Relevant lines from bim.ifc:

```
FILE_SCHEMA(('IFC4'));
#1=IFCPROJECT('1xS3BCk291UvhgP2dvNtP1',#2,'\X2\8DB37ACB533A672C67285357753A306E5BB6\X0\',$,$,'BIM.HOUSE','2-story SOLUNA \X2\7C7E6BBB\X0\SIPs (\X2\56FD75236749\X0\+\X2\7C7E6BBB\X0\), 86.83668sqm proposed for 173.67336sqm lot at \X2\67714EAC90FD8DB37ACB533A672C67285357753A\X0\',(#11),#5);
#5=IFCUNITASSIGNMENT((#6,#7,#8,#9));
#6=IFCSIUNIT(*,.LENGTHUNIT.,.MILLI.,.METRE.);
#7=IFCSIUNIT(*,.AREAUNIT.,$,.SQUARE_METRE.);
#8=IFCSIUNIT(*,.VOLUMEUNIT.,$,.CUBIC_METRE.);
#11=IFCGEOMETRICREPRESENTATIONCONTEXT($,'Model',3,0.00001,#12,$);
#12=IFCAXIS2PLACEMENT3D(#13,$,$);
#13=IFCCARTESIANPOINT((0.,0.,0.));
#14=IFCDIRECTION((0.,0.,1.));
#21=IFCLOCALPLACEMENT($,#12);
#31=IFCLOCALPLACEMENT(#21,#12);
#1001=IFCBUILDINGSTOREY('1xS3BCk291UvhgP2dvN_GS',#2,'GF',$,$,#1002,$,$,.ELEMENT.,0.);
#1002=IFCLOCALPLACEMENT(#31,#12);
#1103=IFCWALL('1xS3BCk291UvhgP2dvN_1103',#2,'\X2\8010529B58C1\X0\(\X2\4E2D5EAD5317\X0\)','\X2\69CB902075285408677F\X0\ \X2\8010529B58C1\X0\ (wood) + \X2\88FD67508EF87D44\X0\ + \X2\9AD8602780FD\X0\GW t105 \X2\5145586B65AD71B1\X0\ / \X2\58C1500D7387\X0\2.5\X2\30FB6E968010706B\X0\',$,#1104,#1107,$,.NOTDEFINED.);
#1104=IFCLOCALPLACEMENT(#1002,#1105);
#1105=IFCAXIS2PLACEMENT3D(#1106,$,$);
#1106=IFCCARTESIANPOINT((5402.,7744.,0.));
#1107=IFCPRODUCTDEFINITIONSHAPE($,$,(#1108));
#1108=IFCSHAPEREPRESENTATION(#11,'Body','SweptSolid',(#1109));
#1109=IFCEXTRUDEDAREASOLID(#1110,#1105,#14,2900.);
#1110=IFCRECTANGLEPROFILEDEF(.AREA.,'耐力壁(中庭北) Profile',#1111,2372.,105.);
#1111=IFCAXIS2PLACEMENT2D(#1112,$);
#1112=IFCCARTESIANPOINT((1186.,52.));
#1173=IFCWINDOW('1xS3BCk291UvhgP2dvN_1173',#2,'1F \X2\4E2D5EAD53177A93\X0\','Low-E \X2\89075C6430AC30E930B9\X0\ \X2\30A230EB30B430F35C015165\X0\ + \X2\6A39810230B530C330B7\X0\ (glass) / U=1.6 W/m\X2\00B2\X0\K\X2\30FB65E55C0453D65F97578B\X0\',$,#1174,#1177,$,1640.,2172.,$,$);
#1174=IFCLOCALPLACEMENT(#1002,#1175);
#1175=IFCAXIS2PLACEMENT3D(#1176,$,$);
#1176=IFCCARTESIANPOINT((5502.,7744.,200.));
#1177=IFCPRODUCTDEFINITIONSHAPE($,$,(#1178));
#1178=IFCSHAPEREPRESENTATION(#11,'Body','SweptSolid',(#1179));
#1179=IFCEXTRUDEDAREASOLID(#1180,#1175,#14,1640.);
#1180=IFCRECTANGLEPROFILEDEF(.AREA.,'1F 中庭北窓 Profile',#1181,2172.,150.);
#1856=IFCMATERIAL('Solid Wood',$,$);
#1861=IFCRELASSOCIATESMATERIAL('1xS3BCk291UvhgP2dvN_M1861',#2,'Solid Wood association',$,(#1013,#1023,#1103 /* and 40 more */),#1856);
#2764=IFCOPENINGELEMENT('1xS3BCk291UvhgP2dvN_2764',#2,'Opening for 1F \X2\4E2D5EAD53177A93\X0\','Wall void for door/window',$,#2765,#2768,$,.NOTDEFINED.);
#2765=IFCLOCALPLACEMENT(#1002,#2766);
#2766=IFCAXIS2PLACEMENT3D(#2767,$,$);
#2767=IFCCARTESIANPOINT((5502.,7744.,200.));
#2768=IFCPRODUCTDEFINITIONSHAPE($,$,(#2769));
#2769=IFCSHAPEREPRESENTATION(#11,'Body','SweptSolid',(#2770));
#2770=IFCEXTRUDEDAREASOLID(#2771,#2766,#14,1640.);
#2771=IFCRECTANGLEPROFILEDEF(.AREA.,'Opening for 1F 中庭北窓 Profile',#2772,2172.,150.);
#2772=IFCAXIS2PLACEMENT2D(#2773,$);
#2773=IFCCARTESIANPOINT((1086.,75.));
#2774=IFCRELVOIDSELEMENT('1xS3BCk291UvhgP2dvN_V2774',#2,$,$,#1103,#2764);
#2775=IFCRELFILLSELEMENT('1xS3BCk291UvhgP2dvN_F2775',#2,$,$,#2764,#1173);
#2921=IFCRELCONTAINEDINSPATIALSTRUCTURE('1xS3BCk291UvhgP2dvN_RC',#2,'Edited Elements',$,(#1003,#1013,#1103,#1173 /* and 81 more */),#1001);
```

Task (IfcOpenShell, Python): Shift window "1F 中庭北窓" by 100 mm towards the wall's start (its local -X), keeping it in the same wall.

```python
import ifcopenshell
import ifcopenshell.api.geometry
import ifcopenshell.util.placement

model = ifcopenshell.open("bim.ifc")

window = model.by_guid("1xS3BCk291UvhgP2dvN_1173")
opening = window.FillsVoids[0].RelatingOpeningElement
wall = opening.VoidsElements[0].RelatingBuildingElement

wall_matrix = ifcopenshell.util.placement.get_local_placement(wall.ObjectPlacement)
shift = wall_matrix[:3, 0] * -100.0
before = ifcopenshell.util.placement.get_local_placement(window.ObjectPlacement)[:3, 3].copy()

# The window is not placed relative to its opening, so move both.
for product in (opening, window):
    matrix = ifcopenshell.util.placement.get_local_placement(product.ObjectPlacement)
    matrix[:3, 3] += shift
    ifcopenshell.api.geometry.edit_object_placement(model, product=product, matrix=matrix, is_si=False)

after = ifcopenshell.util.placement.get_local_placement(window.ObjectPlacement)[:3, 3]
print("window moved by", (after - before).round(3) + 0.0)

model.write("bim_edited.ifc")
```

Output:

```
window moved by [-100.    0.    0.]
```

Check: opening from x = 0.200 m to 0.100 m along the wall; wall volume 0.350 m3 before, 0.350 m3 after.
